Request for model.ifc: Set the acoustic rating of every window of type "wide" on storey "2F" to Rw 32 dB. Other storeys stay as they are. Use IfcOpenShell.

First a look at what the model holds.

```python
import ifcopenshell
import ifcopenshell.util.element

model = ifcopenshell.open("model.ifc")
print(model.schema)
storey = next(s for s in model.by_type("IfcBuildingStorey") if s.Name == "2F")
windows = [e for e in ifcopenshell.util.element.get_decomposition(storey) if e.is_a("IfcWindow")]
seen = {}
for e in windows:
    element_type = ifcopenshell.util.element.get_type(e)
    key = (element_type.Name if element_type != e and element_type else None, ifcopenshell.util.element.get_pset(e, "Pset_WindowCommon", "AcousticRating"))
    seen[key] = seen.get(key, 0) + 1
for (name, value), count in sorted(seen.items(), key=str):
    print(count, "x", name, "|", value)
```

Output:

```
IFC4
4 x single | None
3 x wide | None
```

```python
import ifcopenshell
import ifcopenshell.api.pset
import ifcopenshell.util.element

model = ifcopenshell.open("model.ifc")

storey = next(s for s in model.by_type("IfcBuildingStorey") if s.Name == "2F")
windows = [e for e in ifcopenshell.util.element.get_decomposition(storey) if e.is_a("IfcWindow")]

count = 0
for e in windows:
    element_type = ifcopenshell.util.element.get_type(e)
    if element_type in (None, e) or element_type.Name != "wide":
        continue
    # add_pset returns the element's existing set when there is one.
    pset = ifcopenshell.api.pset.add_pset(model, product=e, name="Pset_WindowCommon")
    ifcopenshell.api.pset.edit_pset(model, pset=pset, properties={"AcousticRating": "Rw 32 dB"})
    count += 1

print(count, "windows updated")

model.write("model_updated.ifc")
```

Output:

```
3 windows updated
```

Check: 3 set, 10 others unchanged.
